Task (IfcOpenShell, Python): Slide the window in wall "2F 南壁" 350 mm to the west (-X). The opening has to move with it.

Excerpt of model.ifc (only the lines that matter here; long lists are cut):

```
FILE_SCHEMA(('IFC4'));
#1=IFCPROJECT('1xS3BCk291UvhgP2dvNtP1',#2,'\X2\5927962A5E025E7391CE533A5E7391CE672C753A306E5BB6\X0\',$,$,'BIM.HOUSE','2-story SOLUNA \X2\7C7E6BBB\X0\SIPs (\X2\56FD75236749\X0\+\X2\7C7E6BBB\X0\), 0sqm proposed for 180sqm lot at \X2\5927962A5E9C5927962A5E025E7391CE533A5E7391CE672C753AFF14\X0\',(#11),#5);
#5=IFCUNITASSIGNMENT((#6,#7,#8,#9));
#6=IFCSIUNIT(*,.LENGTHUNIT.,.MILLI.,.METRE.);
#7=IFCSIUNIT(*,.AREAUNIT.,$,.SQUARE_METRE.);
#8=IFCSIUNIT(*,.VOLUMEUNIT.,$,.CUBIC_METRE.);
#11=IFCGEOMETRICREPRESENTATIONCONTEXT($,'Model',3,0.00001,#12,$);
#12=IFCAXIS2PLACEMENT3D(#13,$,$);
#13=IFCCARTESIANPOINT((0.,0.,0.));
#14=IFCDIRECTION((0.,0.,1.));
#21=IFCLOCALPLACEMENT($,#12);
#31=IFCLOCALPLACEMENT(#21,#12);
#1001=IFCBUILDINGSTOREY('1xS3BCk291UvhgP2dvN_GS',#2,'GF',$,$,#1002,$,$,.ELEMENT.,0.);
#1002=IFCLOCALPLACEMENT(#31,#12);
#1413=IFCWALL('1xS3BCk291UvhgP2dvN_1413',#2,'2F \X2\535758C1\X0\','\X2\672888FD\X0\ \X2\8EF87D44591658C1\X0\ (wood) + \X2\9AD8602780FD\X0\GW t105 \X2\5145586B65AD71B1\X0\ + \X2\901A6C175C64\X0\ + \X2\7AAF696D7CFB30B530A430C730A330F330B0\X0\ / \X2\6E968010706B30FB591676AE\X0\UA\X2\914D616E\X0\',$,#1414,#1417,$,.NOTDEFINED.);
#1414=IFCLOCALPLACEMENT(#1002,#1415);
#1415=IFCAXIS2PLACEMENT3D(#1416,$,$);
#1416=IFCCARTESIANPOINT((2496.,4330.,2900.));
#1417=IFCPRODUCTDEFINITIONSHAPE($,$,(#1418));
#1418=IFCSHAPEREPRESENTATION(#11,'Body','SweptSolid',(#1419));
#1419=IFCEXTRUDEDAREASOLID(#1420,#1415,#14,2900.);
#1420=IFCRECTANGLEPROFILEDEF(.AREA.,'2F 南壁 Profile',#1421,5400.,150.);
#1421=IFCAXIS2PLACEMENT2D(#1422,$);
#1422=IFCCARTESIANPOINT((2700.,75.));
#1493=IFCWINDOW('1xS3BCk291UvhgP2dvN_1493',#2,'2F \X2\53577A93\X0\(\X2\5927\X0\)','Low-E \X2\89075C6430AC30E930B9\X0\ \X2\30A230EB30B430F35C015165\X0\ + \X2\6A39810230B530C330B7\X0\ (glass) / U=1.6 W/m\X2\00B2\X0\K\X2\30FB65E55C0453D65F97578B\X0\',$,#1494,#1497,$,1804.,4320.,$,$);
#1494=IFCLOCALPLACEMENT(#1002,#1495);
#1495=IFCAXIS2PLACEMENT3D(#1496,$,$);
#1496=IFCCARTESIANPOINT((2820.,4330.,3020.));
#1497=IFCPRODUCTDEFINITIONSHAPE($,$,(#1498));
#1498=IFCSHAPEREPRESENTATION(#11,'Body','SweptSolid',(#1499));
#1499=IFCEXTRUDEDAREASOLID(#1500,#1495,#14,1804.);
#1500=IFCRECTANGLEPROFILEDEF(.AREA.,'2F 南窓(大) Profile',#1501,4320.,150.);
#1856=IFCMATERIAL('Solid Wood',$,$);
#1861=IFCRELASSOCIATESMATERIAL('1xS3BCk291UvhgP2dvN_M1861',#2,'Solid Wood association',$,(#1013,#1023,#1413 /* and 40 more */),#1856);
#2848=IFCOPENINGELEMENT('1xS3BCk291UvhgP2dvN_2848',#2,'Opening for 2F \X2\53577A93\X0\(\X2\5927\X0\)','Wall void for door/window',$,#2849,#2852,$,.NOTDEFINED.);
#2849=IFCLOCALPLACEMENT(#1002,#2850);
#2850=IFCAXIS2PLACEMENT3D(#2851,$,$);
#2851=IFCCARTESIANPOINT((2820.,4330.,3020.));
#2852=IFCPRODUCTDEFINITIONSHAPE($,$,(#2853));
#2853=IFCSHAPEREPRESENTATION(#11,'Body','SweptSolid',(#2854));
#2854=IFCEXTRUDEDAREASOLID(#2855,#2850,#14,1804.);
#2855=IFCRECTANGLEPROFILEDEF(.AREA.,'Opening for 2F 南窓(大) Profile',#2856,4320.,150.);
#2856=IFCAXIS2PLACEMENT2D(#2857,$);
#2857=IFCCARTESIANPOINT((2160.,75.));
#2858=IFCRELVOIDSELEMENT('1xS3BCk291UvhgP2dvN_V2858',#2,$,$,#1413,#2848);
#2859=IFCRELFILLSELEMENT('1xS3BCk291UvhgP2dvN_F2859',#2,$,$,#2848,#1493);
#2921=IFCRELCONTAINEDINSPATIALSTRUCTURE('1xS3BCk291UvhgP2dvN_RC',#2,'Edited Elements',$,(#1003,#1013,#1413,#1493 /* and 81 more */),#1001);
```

```python
import ifcopenshell
import ifcopenshell.api.geometry
import ifcopenshell.util.placement
import ifcopenshell.util.unit

model = ifcopenshell.open("model.ifc")
unit_scale = ifcopenshell.util.unit.calculate_unit_scale(model)

window = model.by_guid("1xS3BCk291UvhgP2dvN_1493")
opening = window.FillsVoids[0].RelatingOpeningElement
wall = opening.VoidsElements[0].RelatingBuildingElement

wall_matrix = ifcopenshell.util.placement.get_local_placement(wall.ObjectPlacement)
shift = wall_matrix[:3, 0] * -0.35 / unit_scale
before = ifcopenshell.util.placement.get_local_placement(window.ObjectPlacement)[:3, 3].copy()

# The window is not placed relative to its opening, so move both.
for product in (opening, window):
    matrix = ifcopenshell.util.placement.get_local_placement(product.ObjectPlacement)
    matrix[:3, 3] += shift
    ifcopenshell.api.geometry.edit_object_placement(model, product=product, matrix=matrix, is_si=False)

after = ifcopenshell.util.placement.get_local_placement(window.ObjectPlacement)[:3, 3]
print("window moved by", (after - before).round(3) + 0.0)

model.write("model_edited.ifc")
```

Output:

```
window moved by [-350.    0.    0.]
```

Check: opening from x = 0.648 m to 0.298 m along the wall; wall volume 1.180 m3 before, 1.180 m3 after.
